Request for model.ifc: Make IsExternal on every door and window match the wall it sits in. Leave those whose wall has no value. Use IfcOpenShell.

First a look at what the model holds.

```python
import ifcopenshell
import ifcopenshell.util.element

model = ifcopenshell.open("model.ifc")
print(model.schema)
seen = {}
for e in model.by_type("IfcDoor") + model.by_type("IfcWindow"):
    if not e.FillsVoids:
        continue
    host = e.FillsVoids[0].RelatingOpeningElement.VoidsElements[0].RelatingBuildingElement
    own = ifcopenshell.util.element.get_pset(e, f"Pset_{e.is_a()[3:].removesuffix('StandardCase')}Common", "IsExternal")
    wall = ifcopenshell.util.element.get_pset(host, "Pset_WallCommon", "IsExternal")
    seen[e.is_a(), own, wall] = seen.get((e.is_a(), own, wall), 0) + 1
for (cls, own, wall), count in sorted(seen.items(), key=str):
    print(count, cls, "IsExternal:", own, "| host wall:", wall)
```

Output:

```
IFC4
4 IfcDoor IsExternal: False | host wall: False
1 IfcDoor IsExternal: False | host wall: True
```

```python
import ifcopenshell
import ifcopenshell.api.pset
import ifcopenshell.util.element

model = ifcopenshell.open("model.ifc")

count = 0
for ifc_class, pset_name in (("IfcDoor", "Pset_DoorCommon"), ("IfcWindow", "Pset_WindowCommon")):
    for e in model.by_type(ifc_class):
        if not e.FillsVoids:
            continue
        host = e.FillsVoids[0].RelatingOpeningElement.VoidsElements[0].RelatingBuildingElement
        external = ifcopenshell.util.element.get_pset(host, "Pset_WallCommon", "IsExternal")
        if external is None or ifcopenshell.util.element.get_pset(e, pset_name, "IsExternal") == external:
            continue
        pset = ifcopenshell.api.pset.add_pset(model, product=e, name=pset_name)
        ifcopenshell.api.pset.edit_pset(model, pset=pset, properties={"IsExternal": external})
        count += 1

print(count, "updated")

model.write("model_edited.ifc")
```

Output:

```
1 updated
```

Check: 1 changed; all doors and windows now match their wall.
